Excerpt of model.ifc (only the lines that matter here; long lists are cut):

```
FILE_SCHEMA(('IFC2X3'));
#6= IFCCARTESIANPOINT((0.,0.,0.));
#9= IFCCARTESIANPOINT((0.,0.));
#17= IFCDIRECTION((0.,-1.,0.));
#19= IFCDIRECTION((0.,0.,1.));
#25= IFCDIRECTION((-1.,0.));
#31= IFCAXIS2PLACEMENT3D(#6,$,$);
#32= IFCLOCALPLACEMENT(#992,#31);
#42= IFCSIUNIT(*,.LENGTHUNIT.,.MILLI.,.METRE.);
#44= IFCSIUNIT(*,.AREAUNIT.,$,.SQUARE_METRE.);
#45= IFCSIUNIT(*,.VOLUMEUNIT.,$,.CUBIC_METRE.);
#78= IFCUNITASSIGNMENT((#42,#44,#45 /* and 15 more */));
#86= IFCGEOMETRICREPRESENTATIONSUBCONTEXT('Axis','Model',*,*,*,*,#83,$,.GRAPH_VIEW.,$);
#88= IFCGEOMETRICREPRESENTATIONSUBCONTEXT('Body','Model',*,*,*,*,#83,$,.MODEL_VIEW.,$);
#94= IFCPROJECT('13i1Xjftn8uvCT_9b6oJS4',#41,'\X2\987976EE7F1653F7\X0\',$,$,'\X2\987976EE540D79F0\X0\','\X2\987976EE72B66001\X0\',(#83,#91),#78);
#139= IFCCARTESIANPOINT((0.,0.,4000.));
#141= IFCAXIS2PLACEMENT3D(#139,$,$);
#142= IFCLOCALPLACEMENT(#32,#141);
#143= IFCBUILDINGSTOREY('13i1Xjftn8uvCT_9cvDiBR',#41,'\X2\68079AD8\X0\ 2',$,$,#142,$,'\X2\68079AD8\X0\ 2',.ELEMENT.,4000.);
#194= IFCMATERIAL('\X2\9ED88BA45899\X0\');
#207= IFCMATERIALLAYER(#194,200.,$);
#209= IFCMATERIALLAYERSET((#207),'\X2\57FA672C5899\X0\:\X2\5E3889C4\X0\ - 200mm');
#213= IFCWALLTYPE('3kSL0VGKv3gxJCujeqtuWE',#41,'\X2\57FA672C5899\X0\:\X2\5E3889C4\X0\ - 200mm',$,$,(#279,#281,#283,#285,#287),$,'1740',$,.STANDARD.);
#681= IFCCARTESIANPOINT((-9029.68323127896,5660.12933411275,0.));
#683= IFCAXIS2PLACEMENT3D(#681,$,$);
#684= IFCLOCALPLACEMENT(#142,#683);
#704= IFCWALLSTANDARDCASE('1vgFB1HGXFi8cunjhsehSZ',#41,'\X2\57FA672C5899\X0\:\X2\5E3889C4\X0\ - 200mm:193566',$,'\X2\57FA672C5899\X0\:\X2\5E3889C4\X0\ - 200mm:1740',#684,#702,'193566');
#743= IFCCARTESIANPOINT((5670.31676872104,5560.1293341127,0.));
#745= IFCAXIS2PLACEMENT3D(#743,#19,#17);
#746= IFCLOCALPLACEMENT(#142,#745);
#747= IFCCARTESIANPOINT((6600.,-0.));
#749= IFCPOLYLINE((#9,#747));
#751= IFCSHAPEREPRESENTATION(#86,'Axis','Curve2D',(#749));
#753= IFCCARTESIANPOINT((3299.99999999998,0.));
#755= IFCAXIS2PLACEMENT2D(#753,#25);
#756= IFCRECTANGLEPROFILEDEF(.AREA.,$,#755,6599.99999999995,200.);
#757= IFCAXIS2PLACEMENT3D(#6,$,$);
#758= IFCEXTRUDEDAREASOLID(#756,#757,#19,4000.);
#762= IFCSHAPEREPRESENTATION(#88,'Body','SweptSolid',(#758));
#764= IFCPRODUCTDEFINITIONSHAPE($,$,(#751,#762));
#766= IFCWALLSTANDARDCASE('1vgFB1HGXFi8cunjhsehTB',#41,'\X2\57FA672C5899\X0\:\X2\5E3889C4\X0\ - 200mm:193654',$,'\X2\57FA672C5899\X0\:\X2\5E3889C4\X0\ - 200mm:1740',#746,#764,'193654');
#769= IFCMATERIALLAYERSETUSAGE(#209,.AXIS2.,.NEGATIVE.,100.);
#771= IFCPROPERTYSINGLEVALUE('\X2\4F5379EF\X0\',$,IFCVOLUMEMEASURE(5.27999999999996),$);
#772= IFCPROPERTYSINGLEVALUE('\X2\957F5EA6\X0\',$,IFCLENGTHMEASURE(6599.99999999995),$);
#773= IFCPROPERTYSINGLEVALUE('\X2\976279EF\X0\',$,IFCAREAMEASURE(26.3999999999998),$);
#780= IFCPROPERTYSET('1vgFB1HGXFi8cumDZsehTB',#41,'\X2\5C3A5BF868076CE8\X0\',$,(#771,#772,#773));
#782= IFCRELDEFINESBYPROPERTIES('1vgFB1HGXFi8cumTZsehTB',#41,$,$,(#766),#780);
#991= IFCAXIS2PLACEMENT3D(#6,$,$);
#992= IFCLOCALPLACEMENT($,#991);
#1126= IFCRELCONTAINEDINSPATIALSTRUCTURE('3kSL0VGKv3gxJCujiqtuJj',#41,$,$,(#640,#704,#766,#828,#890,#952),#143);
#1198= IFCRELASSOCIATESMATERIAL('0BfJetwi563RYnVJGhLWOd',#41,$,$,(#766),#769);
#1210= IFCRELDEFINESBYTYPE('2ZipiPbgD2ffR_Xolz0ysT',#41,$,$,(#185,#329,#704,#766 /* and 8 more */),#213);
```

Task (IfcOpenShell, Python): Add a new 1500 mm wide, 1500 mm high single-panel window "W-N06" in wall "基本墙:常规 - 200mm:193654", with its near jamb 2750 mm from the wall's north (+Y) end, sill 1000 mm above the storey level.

```python
import numpy as np
import ifcopenshell
import ifcopenshell.api.feature
import ifcopenshell.api.geometry
import ifcopenshell.api.pset
import ifcopenshell.api.root
import ifcopenshell.api.spatial
import ifcopenshell.api.type
import ifcopenshell.geom
import ifcopenshell.util.element
import ifcopenshell.util.placement
import ifcopenshell.util.representation
import ifcopenshell.util.shape
import ifcopenshell.util.unit

model = ifcopenshell.open("model.ifc")
unit_scale = ifcopenshell.util.unit.calculate_unit_scale(model)
area_scale = ifcopenshell.util.unit.calculate_unit_scale(model, "AREAUNIT")
volume_scale = ifcopenshell.util.unit.calculate_unit_scale(model, "VOLUMEUNIT")
settings = ifcopenshell.geom.settings()


def volume(element):
    """Net volume in cubic metres, openings subtracted."""
    shape = ifcopenshell.geom.create_shape(settings, element)
    return ifcopenshell.util.shape.get_volume(shape.geometry)


wall = model.by_guid("1vgFB1HGXFi8cunjhsehTB")
storey = ifcopenshell.util.element.get_container(wall, ifc_class="IfcBuildingStorey")
context = ifcopenshell.util.representation.get_context(model, "Model", "Body", "MODEL_VIEW")
before = volume(wall)

width, height, from_end, sill = 1.5, 1.5, 2.75, 1  # metres

# The wall runs along its own X axis, and the end named is its -X end.
wall_shape = ifcopenshell.geom.create_shape(settings, wall)
x, y, z = ifcopenshell.util.shape.get_vertices(wall_shape.geometry).T
start = x.min() + from_end
face, thickness = float(y.min()), float(y.max() - y.min())
wall_matrix = ifcopenshell.util.placement.get_local_placement(wall.ObjectPlacement)
level = ifcopenshell.util.placement.get_local_placement(storey.ObjectPlacement)[2, 3]


def in_wall(x, y):
    """Placement at x, y metres in the wall's axes, at sill height."""
    matrix = wall_matrix.copy()
    matrix[:, 3] = wall_matrix @ np.array([x / unit_scale, y / unit_scale, 0.0, 1.0])
    matrix[2, 3] = level + sill / unit_scale
    return matrix


# Opening: a box that overshoots both wall faces by 50 mm.
opening = ifcopenshell.api.root.create_entity(model, ifc_class="IfcOpeningElement")
box = ifcopenshell.api.geometry.add_wall_representation(
    model, context=context, length=width, height=height, thickness=thickness + 0.1
)
ifcopenshell.api.geometry.assign_representation(model, product=opening, representation=box)
ifcopenshell.api.geometry.edit_object_placement(model, product=opening, matrix=in_wall(start, face - 0.05), is_si=False)
ifcopenshell.api.feature.add_feature(model, feature=opening, element=wall)

window = ifcopenshell.api.root.create_entity(model, ifc_class="IfcWindow", name="W-N06")
window.OverallWidth, window.OverallHeight = width / unit_scale, height / unit_scale
body = ifcopenshell.api.geometry.add_window_representation(
    model,
    context=context,
    overall_width=window.OverallWidth,
    overall_height=window.OverallHeight,
    partition_type="SINGLE_PANEL",
)
ifcopenshell.api.geometry.assign_representation(model, product=window, representation=body)
ifcopenshell.api.spatial.assign_container(model, products=[window], relating_structure=storey)
fills = ifcopenshell.api.feature.add_filling(model, opening=opening, element=window)
fills.OwnerHistory = window.OwnerHistory  # required in IFC2X3

# IFC2X3 keeps the operation on the window style.
style = ifcopenshell.api.root.create_entity(model, ifc_class="IfcWindowStyle", name="W-N06")
style.OperationType, style.ConstructionType = "SINGLE_PANEL", "NOTDEFINED"
style.ParameterTakesPrecedence = style.Sizeable = False
ifcopenshell.api.type.assign_type(model, related_objects=[window], relating_type=style)

# Centre the window in the wall's thickness.
ifcopenshell.api.geometry.edit_object_placement(model, product=window, matrix=in_wall(start, face), is_si=False)
window_shape = ifcopenshell.geom.create_shape(settings, window)
depth = ifcopenshell.util.shape.get_vertices(window_shape.geometry)[:, 1]
offset = face + thickness / 2 - (depth.min() + depth.max()) / 2
ifcopenshell.api.geometry.edit_object_placement(model, product=window, matrix=in_wall(start, offset), is_si=False)

after = volume(wall)

# Update the wall's stored quantities.
pset = model.by_id(ifcopenshell.util.element.get_pset(wall, "尺寸标注", should_inherit=False)["id"])
ifcopenshell.api.pset.edit_pset(model, pset=pset, properties={
    "体积": model.create_entity("IfcVolumeMeasure", after / volume_scale),
    "面积": model.create_entity("IfcAreaMeasure", after / thickness / area_scale),
})

print(f"wall volume {before:.3f} -> {after:.3f} m3")

model.write("model_updated.ifc")
```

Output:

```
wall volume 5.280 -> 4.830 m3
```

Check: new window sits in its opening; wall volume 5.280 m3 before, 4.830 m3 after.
